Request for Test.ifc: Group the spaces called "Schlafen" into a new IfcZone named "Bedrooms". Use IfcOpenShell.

First a look at what the model holds.

```python
import ifcopenshell

model = ifcopenshell.open("Test.ifc")
print(model.schema)
seen = {}
for space in model.by_type("IfcSpace"):
    seen[space.LongName] = seen.get(space.LongName, 0) + 1
for name, count in sorted(seen.items(), key=str):
    print(count, "x", name)
print("zones:", [z.Name for z in model.by_type("IfcZone")][:20])
```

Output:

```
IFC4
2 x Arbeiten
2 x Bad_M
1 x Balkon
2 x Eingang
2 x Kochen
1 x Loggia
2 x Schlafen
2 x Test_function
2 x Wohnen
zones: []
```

```python
import ifcopenshell
import ifcopenshell.api.group
import ifcopenshell.api.root

model = ifcopenshell.open("Test.ifc")

names = {"Schlafen"}
spaces = [s for s in model.by_type("IfcSpace") if s.LongName in names]

zone = ifcopenshell.api.root.create_entity(model, ifc_class="IfcZone", name="Bedrooms")
ifcopenshell.api.group.assign_group(model, products=spaces, group=zone)
print(len(spaces), "spaces in", zone.Name)

model.write("Test_edited.ifc")
```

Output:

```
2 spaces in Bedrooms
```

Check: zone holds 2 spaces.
